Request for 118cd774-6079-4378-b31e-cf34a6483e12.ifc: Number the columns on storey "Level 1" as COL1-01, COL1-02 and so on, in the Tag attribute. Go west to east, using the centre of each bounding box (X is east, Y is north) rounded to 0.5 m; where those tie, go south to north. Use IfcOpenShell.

First a look at what the model holds.

```python
import ifcopenshell
import ifcopenshell.util.element
import ifcopenshell.util.placement

model = ifcopenshell.open("118cd774-6079-4378-b31e-cf34a6483e12.ifc")
print(model.schema)
storey = next(s for s in model.by_type("IfcBuildingStorey") if s.Name == "Level 1")
columns = [e for e in ifcopenshell.util.element.get_decomposition(storey) if e.is_a("IfcColumn")]
for e in sorted(columns, key=lambda e: e.id()):
    origin = ifcopenshell.util.placement.get_local_placement(e.ObjectPlacement)[:3, 3]
    print(e.id(), e.Tag, e.Name, origin.round(2) + 0.0, sep=" | ")
```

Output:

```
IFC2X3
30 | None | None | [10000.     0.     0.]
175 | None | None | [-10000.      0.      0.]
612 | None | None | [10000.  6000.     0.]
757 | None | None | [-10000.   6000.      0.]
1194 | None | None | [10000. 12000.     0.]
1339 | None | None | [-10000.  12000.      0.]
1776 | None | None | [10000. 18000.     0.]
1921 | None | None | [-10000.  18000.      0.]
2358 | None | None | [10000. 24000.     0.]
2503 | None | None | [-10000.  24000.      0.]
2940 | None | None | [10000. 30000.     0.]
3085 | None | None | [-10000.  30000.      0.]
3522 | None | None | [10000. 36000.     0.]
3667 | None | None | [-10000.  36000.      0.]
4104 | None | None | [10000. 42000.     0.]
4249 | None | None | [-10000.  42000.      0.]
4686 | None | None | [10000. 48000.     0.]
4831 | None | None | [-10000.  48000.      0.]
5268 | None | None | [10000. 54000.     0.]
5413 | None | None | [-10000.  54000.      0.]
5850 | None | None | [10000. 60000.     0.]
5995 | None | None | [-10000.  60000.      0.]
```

```python
import ifcopenshell
import ifcopenshell.geom
import ifcopenshell.util.element
import ifcopenshell.util.shape

model = ifcopenshell.open("118cd774-6079-4378-b31e-cf34a6483e12.ifc")
settings = ifcopenshell.geom.settings()
settings.set("use-world-coords", True)


def centre(element):
    shape = ifcopenshell.geom.create_shape(settings, element)
    return ifcopenshell.util.shape.get_bbox_centroid(shape.geometry)


storey = next(s for s in model.by_type("IfcBuildingStorey") if s.Name == "Level 1")
columns = [e for e in ifcopenshell.util.element.get_decomposition(storey) if e.is_a("IfcColumn")]

# Insertion points can sit at a corner or the storey origin, so sort by the geometry (in metres).
centres = {e: centre(e) for e in columns}
columns.sort(key=lambda e: (round(centres[e][0] / 0.5), centres[e][1]))

for i, e in enumerate(columns, start=1):
    number = f"COL1-{i:02d}"
    e.Tag = number
    print(e.id(), number)

model.write("118cd774-6079-4378-b31e-cf34a6483e12_edited.ifc")
```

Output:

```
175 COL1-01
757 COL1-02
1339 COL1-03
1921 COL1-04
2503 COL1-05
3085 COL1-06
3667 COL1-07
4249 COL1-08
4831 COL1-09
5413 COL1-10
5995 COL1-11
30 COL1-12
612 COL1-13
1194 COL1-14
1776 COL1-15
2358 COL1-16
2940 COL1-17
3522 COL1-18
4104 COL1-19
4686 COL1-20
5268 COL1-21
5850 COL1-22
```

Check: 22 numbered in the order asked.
